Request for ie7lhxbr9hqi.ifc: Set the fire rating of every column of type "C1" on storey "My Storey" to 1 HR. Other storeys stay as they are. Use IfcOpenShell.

First a look at what the model holds.

```python
import ifcopenshell
import ifcopenshell.util.element

model = ifcopenshell.open("ie7lhxbr9hqi.ifc")
print(model.schema)
storey = next(s for s in model.by_type("IfcBuildingStorey") if s.Name == "My Storey")
columns = [e for e in ifcopenshell.util.element.get_decomposition(storey) if e.is_a("IfcColumn")]
seen = {}
for e in columns:
    element_type = ifcopenshell.util.element.get_type(e)
    key = (element_type.Name if element_type != e and element_type else None, ifcopenshell.util.element.get_pset(e, "Pset_ColumnCommon", "FireRating"))
    seen[key] = seen.get(key, 0) + 1
for (name, value), count in sorted(seen.items(), key=str):
    print(count, "x", name, "|", value)
```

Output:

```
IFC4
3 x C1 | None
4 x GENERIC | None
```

```python
import ifcopenshell
import ifcopenshell.api.pset
import ifcopenshell.util.element

model = ifcopenshell.open("ie7lhxbr9hqi.ifc")

storey = next(s for s in model.by_type("IfcBuildingStorey") if s.Name == "My Storey")
columns = [e for e in ifcopenshell.util.element.get_decomposition(storey) if e.is_a("IfcColumn")]

count = 0
for e in columns:
    element_type = ifcopenshell.util.element.get_type(e)
    if element_type in (None, e) or element_type.Name != "C1":
        continue
    # add_pset returns the element's existing set when there is one.
    pset = ifcopenshell.api.pset.add_pset(model, product=e, name="Pset_ColumnCommon")
    ifcopenshell.api.pset.edit_pset(model, pset=pset, properties={"FireRating": "1 HR"})
    count += 1

print(count, "columns updated")

model.write("ie7lhxbr9hqi-out.ifc")
```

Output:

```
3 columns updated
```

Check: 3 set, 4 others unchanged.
